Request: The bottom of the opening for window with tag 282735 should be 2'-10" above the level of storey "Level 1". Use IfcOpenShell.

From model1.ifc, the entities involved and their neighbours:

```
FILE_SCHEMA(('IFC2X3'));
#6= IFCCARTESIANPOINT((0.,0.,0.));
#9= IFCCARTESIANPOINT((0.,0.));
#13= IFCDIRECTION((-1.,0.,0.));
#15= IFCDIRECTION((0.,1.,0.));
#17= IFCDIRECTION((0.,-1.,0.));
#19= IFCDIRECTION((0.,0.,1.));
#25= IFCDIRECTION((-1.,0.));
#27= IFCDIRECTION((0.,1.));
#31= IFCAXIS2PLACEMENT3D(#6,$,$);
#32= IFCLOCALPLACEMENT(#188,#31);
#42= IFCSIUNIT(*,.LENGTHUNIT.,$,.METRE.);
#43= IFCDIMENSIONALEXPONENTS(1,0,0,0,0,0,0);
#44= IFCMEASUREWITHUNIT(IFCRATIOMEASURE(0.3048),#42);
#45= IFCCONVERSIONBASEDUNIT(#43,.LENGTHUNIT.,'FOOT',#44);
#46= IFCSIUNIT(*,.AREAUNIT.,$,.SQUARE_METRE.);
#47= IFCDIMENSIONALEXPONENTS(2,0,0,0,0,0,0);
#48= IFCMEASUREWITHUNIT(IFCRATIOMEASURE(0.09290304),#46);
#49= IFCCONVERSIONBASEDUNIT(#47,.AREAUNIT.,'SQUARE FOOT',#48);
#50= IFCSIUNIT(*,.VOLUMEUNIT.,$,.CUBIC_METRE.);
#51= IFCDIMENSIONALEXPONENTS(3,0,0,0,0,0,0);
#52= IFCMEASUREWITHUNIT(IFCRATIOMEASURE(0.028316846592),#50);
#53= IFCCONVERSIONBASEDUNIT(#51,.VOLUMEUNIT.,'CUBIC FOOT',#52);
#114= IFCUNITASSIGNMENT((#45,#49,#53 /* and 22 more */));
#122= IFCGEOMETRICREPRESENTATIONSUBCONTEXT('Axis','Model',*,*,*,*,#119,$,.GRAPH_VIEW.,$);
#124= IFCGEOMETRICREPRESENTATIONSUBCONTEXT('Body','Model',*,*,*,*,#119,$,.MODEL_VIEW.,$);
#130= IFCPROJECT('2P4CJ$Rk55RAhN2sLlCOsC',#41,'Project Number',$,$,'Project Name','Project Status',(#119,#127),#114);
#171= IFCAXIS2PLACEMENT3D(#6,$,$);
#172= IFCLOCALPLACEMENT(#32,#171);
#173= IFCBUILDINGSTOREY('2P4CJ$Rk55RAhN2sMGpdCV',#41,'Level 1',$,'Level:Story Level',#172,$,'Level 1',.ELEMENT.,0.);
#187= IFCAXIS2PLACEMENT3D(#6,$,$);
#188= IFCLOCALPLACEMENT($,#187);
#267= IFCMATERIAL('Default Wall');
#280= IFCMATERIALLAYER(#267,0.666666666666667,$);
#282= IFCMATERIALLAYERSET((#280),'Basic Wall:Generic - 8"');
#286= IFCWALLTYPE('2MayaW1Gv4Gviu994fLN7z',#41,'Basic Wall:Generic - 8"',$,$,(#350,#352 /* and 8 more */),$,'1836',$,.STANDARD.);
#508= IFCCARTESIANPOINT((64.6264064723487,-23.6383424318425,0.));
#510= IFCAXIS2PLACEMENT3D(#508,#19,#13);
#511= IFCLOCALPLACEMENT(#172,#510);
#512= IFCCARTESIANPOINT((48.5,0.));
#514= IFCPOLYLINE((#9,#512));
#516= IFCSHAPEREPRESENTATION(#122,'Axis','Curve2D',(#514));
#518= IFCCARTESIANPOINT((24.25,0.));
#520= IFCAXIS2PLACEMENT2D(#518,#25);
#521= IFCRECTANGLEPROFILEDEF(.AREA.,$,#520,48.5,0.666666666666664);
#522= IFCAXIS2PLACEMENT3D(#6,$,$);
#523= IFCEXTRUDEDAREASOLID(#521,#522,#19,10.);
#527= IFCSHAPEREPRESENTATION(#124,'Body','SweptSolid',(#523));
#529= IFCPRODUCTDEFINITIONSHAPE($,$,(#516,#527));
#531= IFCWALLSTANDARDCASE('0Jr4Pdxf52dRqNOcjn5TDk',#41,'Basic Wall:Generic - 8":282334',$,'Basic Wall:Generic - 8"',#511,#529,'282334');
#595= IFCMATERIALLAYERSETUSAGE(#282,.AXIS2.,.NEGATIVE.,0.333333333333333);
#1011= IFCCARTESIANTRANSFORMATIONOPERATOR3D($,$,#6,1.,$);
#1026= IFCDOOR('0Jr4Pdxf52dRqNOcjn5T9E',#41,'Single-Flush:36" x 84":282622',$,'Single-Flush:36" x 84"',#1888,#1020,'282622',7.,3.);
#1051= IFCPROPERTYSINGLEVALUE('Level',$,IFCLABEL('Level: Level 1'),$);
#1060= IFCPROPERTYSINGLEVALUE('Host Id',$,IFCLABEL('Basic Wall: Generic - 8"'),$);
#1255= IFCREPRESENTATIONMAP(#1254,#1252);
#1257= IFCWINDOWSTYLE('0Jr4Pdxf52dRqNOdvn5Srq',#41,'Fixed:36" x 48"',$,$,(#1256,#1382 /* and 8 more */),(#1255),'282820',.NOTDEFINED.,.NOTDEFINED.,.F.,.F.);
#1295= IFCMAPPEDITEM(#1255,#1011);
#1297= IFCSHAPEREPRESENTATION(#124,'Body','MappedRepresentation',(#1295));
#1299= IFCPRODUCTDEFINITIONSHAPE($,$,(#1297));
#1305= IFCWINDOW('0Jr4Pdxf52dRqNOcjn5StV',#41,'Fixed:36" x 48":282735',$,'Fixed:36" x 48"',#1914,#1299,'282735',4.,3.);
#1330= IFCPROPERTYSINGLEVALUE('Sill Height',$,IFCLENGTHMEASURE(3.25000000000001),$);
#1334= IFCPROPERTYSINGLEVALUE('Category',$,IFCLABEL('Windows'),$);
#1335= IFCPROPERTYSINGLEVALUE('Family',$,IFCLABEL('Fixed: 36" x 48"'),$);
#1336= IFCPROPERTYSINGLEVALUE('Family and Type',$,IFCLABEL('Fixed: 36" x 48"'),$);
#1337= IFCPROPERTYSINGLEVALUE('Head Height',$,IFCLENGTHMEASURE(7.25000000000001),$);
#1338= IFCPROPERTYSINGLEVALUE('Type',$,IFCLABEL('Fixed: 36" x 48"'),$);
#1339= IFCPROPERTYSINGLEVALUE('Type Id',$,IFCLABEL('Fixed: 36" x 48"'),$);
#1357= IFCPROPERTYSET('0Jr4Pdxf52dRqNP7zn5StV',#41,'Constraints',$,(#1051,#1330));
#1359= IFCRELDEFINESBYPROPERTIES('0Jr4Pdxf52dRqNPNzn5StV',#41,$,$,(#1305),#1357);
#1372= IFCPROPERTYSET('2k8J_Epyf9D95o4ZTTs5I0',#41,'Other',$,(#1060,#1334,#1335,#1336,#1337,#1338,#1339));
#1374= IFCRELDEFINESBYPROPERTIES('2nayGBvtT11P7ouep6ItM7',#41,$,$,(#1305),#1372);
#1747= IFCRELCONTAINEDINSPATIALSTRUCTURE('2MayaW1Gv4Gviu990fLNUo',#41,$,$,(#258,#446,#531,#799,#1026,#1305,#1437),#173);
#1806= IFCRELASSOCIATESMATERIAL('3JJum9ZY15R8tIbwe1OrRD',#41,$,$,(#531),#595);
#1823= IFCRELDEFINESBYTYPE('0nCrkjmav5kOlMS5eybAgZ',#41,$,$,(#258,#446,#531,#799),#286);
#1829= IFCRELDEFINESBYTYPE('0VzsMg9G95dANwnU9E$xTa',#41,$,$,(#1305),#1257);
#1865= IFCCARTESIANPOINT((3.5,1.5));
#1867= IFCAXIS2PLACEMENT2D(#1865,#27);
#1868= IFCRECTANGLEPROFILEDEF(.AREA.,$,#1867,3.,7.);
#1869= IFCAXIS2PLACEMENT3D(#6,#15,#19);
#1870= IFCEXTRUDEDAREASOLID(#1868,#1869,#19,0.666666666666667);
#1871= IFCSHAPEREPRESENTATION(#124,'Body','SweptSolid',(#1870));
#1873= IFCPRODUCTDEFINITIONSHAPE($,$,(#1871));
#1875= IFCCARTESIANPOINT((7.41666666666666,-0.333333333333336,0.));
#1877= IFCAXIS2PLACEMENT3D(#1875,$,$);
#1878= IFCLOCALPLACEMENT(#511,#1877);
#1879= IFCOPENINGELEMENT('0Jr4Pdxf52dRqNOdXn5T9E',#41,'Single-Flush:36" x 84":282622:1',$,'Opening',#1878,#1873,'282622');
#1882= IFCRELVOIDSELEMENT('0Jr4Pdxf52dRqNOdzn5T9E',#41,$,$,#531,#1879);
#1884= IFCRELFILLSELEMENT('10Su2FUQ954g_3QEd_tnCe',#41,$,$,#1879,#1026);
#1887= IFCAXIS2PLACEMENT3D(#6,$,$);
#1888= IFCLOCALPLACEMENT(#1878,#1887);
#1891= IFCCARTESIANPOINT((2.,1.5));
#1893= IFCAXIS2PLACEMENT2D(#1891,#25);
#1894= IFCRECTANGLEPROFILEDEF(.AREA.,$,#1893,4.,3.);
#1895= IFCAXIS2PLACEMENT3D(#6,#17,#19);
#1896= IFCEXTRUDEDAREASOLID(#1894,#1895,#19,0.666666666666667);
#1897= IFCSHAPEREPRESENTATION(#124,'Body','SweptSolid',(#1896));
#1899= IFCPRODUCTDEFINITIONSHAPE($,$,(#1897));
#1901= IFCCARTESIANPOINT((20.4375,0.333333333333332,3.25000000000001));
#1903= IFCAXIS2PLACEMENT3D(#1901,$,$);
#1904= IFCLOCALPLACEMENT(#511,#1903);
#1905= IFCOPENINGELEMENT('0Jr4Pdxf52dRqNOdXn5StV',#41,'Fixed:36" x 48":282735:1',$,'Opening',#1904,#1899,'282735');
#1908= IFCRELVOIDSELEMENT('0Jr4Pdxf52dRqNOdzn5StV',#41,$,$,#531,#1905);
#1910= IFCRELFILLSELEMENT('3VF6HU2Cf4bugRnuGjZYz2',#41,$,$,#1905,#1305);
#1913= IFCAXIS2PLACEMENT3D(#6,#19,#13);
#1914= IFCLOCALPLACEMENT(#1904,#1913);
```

```python
import numpy as np
import ifcopenshell
import ifcopenshell.api.geometry
import ifcopenshell.api.pset
import ifcopenshell.geom
import ifcopenshell.util.element
import ifcopenshell.util.placement
import ifcopenshell.util.shape
import ifcopenshell.util.unit

model = ifcopenshell.open("model1.ifc")
unit_scale = ifcopenshell.util.unit.calculate_unit_scale(model)

window = model.by_guid("0Jr4Pdxf52dRqNOcjn5StV")
opening = window.FillsVoids[0].RelatingOpeningElement
storey = ifcopenshell.util.element.get_container(window, ifc_class="IfcBuildingStorey")
level = ifcopenshell.util.placement.get_local_placement(storey.ObjectPlacement)[2, 3]

# The opening's origin need not be at the sill, so measure its lowest point.
shape = ifcopenshell.geom.create_shape(ifcopenshell.geom.settings(), opening)
bottom = ifcopenshell.util.shape.get_shape_bottom_elevation(shape, shape.geometry) / unit_scale
dz = level + 34 * 0.0254 / unit_scale - bottom

shift = np.array([0.0, 0.0, dz])
# The window is placed relative to its opening, so it follows when the opening moves.
matrix = ifcopenshell.util.placement.get_local_placement(opening.ObjectPlacement)
matrix[:3, 3] += shift
ifcopenshell.api.geometry.edit_object_placement(
    model, product=opening, matrix=matrix, is_si=False, should_transform_children=True
)

# Keep the stored heights in step.
pset = model.by_id(ifcopenshell.util.element.get_pset(window, "Constraints", should_inherit=False)["id"])
ifcopenshell.api.pset.edit_pset(model, pset=pset, properties={
    "Sill Height": model.create_entity("IfcLengthMeasure", ifcopenshell.util.element.get_pset(window, "Constraints", "Sill Height") + dz),
})
pset = model.by_id(ifcopenshell.util.element.get_pset(window, "Other", should_inherit=False)["id"])
ifcopenshell.api.pset.edit_pset(model, pset=pset, properties={
    "Head Height": model.create_entity("IfcLengthMeasure", ifcopenshell.util.element.get_pset(window, "Other", "Head Height") + dz),
})

print(f"moved by {dz * unit_scale:+.3f} m")

model.write("model1_v2.ifc")
```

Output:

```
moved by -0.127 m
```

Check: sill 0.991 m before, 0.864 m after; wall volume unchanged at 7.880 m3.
